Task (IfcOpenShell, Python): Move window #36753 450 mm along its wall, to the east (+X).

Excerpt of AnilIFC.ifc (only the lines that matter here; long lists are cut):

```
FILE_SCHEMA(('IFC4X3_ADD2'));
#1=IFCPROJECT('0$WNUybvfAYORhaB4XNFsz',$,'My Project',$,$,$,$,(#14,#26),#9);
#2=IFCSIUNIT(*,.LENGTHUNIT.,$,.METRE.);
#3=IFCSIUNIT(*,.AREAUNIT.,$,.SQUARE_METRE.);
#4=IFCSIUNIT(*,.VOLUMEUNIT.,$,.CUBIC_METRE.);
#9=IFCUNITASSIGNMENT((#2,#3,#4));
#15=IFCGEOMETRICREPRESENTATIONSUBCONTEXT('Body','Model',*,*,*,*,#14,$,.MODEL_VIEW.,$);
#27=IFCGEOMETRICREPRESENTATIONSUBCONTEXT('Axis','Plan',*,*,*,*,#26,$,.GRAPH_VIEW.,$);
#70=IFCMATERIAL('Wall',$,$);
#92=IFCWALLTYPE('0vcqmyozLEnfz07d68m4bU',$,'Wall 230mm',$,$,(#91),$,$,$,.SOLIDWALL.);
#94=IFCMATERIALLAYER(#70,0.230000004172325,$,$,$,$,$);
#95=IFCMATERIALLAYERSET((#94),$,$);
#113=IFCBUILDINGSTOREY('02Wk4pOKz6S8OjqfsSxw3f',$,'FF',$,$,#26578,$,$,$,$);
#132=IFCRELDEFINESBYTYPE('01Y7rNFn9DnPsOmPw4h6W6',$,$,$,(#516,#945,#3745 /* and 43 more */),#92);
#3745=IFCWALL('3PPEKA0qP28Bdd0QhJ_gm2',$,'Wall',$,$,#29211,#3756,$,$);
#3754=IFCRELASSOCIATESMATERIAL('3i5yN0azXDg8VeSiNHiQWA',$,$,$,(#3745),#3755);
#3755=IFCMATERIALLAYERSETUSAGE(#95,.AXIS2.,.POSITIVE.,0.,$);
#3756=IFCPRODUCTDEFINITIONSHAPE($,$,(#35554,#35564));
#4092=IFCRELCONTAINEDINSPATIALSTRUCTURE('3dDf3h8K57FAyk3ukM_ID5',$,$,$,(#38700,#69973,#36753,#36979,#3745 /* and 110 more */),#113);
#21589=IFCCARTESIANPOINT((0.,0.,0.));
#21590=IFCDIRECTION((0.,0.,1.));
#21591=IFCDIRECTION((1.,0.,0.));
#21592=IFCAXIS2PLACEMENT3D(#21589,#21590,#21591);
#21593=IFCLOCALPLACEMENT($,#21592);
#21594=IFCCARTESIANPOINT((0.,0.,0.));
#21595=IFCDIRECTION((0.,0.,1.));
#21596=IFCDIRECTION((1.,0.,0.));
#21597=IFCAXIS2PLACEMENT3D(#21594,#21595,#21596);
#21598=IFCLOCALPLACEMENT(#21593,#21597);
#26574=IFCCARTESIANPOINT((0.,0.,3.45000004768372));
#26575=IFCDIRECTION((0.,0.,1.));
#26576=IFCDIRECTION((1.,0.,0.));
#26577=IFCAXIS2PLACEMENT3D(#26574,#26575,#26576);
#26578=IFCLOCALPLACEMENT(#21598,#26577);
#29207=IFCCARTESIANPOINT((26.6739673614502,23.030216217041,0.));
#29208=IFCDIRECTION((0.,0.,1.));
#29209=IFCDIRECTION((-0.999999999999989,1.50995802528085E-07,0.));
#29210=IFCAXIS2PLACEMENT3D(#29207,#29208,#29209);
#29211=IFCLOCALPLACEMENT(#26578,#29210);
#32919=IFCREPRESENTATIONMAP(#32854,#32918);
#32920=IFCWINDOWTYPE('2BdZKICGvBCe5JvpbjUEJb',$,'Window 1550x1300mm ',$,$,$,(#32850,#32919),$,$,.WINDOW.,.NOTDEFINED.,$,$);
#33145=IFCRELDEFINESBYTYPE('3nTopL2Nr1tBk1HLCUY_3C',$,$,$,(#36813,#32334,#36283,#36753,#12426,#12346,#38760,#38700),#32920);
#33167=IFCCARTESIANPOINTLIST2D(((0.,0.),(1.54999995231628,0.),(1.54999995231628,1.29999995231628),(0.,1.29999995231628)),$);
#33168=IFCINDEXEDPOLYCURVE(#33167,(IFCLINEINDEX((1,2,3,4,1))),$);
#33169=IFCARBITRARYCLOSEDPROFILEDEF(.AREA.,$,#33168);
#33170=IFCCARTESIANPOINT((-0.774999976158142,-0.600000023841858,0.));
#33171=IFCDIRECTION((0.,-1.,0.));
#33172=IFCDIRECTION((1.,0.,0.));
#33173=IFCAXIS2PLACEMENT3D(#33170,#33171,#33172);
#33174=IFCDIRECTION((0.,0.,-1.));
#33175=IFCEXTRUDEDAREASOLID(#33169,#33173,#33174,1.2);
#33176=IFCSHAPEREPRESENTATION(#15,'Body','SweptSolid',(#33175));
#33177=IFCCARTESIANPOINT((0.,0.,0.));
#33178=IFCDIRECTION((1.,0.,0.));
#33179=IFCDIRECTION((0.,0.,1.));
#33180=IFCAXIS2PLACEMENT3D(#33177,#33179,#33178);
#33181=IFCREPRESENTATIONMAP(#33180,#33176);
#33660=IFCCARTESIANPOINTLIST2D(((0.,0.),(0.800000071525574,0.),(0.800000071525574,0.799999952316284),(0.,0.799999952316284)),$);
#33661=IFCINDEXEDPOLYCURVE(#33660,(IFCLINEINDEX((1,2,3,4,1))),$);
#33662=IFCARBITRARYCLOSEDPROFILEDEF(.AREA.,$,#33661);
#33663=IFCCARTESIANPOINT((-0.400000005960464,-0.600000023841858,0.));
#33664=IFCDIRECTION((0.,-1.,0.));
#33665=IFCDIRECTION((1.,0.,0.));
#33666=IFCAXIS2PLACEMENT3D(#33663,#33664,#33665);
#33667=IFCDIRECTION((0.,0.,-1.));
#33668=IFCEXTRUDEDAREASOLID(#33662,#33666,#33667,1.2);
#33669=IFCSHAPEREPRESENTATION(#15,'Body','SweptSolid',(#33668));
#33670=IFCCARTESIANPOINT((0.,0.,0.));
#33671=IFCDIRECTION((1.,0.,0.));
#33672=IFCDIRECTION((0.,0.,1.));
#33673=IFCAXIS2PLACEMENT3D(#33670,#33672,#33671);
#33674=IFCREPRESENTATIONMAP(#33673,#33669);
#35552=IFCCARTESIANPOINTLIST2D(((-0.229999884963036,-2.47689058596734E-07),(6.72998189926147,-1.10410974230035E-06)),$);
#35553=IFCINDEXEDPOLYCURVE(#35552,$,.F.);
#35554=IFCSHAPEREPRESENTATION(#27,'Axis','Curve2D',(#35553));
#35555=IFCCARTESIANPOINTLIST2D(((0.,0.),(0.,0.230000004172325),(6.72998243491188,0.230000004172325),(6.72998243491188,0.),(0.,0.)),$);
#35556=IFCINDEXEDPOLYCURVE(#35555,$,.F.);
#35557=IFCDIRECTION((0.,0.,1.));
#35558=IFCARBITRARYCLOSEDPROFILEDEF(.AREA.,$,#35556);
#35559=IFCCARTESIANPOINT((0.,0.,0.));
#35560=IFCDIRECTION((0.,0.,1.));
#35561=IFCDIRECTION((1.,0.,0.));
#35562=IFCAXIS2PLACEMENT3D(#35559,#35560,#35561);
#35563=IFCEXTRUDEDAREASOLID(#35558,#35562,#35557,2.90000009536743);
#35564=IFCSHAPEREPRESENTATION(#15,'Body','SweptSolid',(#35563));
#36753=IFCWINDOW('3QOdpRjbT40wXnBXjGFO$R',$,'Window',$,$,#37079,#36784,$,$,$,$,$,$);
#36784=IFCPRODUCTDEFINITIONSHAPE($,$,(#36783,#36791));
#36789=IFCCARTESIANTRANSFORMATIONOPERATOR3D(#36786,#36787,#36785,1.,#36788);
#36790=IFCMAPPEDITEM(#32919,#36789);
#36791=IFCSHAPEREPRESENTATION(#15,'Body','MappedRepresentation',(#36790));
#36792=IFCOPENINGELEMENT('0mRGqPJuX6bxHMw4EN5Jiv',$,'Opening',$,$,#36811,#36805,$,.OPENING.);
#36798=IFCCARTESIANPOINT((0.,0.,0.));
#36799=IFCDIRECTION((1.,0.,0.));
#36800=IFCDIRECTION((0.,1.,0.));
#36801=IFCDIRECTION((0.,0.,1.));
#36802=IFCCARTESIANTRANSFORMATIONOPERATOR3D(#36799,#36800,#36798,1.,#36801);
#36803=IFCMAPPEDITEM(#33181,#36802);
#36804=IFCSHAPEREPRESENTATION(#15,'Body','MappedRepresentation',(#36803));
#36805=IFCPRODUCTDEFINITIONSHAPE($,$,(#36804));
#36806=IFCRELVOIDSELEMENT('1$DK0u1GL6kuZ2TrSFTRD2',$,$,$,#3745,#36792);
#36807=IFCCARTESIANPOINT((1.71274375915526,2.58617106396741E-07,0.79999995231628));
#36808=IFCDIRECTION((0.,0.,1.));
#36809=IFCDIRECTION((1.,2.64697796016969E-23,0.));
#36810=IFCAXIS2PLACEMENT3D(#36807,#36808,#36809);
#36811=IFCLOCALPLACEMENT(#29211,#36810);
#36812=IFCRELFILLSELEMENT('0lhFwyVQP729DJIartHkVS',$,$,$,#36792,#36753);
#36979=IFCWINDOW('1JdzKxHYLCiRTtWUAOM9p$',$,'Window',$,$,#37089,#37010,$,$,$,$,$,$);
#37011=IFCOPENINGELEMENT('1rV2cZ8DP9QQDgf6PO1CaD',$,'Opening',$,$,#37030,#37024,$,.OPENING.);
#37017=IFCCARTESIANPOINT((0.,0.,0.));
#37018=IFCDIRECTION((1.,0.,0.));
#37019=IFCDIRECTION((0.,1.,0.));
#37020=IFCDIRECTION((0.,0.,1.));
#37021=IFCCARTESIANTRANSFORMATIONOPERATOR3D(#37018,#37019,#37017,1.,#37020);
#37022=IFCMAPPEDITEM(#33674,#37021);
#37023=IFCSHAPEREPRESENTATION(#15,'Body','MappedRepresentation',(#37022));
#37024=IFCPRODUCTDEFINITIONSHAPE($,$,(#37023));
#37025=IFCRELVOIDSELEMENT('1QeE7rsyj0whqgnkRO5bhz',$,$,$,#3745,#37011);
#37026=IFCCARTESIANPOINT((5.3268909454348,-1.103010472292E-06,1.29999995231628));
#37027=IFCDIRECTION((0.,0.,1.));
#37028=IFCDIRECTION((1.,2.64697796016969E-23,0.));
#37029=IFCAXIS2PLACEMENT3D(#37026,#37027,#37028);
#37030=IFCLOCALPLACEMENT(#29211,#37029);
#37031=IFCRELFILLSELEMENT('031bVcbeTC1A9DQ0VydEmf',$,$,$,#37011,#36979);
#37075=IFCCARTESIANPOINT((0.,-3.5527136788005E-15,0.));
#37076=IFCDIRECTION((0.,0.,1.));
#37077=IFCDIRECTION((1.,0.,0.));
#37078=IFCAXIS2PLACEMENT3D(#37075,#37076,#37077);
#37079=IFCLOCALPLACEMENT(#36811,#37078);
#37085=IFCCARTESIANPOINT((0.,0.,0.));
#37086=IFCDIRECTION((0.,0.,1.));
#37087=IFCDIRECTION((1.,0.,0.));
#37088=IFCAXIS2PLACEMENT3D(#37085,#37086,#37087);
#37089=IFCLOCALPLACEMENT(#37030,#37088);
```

```python
import ifcopenshell
import ifcopenshell.api.geometry
import ifcopenshell.util.placement
import ifcopenshell.util.unit

model = ifcopenshell.open("AnilIFC.ifc")
unit_scale = ifcopenshell.util.unit.calculate_unit_scale(model)

window = model.by_guid("3QOdpRjbT40wXnBXjGFO$R")
opening = window.FillsVoids[0].RelatingOpeningElement
wall = opening.VoidsElements[0].RelatingBuildingElement

wall_matrix = ifcopenshell.util.placement.get_local_placement(wall.ObjectPlacement)
shift = wall_matrix[:3, 0] * -0.45 / unit_scale
before = ifcopenshell.util.placement.get_local_placement(window.ObjectPlacement)[:3, 3].copy()

# The window is placed relative to its opening, so it follows when the opening moves.
matrix = ifcopenshell.util.placement.get_local_placement(opening.ObjectPlacement)
matrix[:3, 3] += shift
ifcopenshell.api.geometry.edit_object_placement(
    model, product=opening, matrix=matrix, is_si=False, should_transform_children=True
)

after = ifcopenshell.util.placement.get_local_placement(window.ObjectPlacement)[:3, 3]
print("window moved by", (after - before).round(3) + 0.0)

model.write("AnilIFC_rev.ifc")
```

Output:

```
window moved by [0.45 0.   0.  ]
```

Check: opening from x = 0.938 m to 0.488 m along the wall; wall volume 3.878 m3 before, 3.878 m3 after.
